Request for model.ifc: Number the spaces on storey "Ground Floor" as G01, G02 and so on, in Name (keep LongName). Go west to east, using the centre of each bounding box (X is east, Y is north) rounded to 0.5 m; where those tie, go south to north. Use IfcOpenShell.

First a look at what the model holds.

```python
import ifcopenshell
import ifcopenshell.util.element
import ifcopenshell.util.placement

model = ifcopenshell.open("model.ifc")
print(model.schema)
storey = next(s for s in model.by_type("IfcBuildingStorey") if s.Name == "Ground Floor")
spaces = [e for e in ifcopenshell.util.element.get_decomposition(storey) if e.is_a("IfcSpace")]
for e in sorted(spaces, key=lambda e: e.id()):
    origin = ifcopenshell.util.placement.get_local_placement(e.ObjectPlacement)[:3, 3]
    print(e.id(), e.Name, e.LongName, origin.round(2) + 0.0, sep=" | ")
```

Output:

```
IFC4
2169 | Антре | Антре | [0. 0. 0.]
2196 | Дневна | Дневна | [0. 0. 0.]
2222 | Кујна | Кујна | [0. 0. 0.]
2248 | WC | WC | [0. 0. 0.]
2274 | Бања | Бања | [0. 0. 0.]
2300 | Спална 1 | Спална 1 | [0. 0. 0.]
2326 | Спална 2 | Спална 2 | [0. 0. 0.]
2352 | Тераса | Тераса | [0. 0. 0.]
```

```python
import ifcopenshell
import ifcopenshell.geom
import ifcopenshell.util.element
import ifcopenshell.util.shape

model = ifcopenshell.open("model.ifc")
settings = ifcopenshell.geom.settings()
settings.set("use-world-coords", True)


def centre(element):
    shape = ifcopenshell.geom.create_shape(settings, element)
    return ifcopenshell.util.shape.get_bbox_centroid(shape.geometry)


storey = next(s for s in model.by_type("IfcBuildingStorey") if s.Name == "Ground Floor")
spaces = [e for e in ifcopenshell.util.element.get_decomposition(storey) if e.is_a("IfcSpace")]

# Insertion points can sit at a corner or the storey origin, so sort by the geometry (in metres).
centres = {e: centre(e) for e in spaces}
spaces.sort(key=lambda e: (round(centres[e][0] / 0.5), centres[e][1]))

for i, e in enumerate(spaces, start=1):
    number = f"G{i:02d}"
    e.Name = number
    print(e.id(), number)

model.write("model_rev.ifc")
```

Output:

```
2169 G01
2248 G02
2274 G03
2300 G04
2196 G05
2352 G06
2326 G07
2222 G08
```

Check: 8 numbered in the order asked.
